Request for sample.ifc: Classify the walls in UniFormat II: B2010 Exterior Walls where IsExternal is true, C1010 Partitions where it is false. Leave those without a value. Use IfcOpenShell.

First a look at what the model holds.

```python
import ifcopenshell
import ifcopenshell.util.element

model = ifcopenshell.open("sample.ifc")
print(model.schema)
print("classifications:", [c.Name for c in model.by_type("IfcClassification")])
values = [ifcopenshell.util.element.get_pset(e, "Pset_WallCommon", "IsExternal") for e in model.by_type("IfcWall")]
for value in (True, False, None):
    print("IsExternal", value, values.count(value))
```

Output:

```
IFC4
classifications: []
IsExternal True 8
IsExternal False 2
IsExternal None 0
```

```python
import ifcopenshell
import ifcopenshell.api.classification
import ifcopenshell.util.element

model = ifcopenshell.open("sample.ifc")

system = ifcopenshell.api.classification.add_classification(model, classification="UniFormat II")

walls = model.by_type("IfcWall")
external = {e: ifcopenshell.util.element.get_pset(e, "Pset_WallCommon", "IsExternal") for e in walls}
for flag, code, name in ((True, "B2010", "Exterior Walls"), (False, "C1010", "Partitions")):
    products = [e for e in walls if external[e] is flag]
    ifcopenshell.api.classification.add_reference(
        model, products=products, classification=system, identification=code, name=name
    )
    print(code, len(products))

model.write("sample-out.ifc")
```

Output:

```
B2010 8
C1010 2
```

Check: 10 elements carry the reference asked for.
